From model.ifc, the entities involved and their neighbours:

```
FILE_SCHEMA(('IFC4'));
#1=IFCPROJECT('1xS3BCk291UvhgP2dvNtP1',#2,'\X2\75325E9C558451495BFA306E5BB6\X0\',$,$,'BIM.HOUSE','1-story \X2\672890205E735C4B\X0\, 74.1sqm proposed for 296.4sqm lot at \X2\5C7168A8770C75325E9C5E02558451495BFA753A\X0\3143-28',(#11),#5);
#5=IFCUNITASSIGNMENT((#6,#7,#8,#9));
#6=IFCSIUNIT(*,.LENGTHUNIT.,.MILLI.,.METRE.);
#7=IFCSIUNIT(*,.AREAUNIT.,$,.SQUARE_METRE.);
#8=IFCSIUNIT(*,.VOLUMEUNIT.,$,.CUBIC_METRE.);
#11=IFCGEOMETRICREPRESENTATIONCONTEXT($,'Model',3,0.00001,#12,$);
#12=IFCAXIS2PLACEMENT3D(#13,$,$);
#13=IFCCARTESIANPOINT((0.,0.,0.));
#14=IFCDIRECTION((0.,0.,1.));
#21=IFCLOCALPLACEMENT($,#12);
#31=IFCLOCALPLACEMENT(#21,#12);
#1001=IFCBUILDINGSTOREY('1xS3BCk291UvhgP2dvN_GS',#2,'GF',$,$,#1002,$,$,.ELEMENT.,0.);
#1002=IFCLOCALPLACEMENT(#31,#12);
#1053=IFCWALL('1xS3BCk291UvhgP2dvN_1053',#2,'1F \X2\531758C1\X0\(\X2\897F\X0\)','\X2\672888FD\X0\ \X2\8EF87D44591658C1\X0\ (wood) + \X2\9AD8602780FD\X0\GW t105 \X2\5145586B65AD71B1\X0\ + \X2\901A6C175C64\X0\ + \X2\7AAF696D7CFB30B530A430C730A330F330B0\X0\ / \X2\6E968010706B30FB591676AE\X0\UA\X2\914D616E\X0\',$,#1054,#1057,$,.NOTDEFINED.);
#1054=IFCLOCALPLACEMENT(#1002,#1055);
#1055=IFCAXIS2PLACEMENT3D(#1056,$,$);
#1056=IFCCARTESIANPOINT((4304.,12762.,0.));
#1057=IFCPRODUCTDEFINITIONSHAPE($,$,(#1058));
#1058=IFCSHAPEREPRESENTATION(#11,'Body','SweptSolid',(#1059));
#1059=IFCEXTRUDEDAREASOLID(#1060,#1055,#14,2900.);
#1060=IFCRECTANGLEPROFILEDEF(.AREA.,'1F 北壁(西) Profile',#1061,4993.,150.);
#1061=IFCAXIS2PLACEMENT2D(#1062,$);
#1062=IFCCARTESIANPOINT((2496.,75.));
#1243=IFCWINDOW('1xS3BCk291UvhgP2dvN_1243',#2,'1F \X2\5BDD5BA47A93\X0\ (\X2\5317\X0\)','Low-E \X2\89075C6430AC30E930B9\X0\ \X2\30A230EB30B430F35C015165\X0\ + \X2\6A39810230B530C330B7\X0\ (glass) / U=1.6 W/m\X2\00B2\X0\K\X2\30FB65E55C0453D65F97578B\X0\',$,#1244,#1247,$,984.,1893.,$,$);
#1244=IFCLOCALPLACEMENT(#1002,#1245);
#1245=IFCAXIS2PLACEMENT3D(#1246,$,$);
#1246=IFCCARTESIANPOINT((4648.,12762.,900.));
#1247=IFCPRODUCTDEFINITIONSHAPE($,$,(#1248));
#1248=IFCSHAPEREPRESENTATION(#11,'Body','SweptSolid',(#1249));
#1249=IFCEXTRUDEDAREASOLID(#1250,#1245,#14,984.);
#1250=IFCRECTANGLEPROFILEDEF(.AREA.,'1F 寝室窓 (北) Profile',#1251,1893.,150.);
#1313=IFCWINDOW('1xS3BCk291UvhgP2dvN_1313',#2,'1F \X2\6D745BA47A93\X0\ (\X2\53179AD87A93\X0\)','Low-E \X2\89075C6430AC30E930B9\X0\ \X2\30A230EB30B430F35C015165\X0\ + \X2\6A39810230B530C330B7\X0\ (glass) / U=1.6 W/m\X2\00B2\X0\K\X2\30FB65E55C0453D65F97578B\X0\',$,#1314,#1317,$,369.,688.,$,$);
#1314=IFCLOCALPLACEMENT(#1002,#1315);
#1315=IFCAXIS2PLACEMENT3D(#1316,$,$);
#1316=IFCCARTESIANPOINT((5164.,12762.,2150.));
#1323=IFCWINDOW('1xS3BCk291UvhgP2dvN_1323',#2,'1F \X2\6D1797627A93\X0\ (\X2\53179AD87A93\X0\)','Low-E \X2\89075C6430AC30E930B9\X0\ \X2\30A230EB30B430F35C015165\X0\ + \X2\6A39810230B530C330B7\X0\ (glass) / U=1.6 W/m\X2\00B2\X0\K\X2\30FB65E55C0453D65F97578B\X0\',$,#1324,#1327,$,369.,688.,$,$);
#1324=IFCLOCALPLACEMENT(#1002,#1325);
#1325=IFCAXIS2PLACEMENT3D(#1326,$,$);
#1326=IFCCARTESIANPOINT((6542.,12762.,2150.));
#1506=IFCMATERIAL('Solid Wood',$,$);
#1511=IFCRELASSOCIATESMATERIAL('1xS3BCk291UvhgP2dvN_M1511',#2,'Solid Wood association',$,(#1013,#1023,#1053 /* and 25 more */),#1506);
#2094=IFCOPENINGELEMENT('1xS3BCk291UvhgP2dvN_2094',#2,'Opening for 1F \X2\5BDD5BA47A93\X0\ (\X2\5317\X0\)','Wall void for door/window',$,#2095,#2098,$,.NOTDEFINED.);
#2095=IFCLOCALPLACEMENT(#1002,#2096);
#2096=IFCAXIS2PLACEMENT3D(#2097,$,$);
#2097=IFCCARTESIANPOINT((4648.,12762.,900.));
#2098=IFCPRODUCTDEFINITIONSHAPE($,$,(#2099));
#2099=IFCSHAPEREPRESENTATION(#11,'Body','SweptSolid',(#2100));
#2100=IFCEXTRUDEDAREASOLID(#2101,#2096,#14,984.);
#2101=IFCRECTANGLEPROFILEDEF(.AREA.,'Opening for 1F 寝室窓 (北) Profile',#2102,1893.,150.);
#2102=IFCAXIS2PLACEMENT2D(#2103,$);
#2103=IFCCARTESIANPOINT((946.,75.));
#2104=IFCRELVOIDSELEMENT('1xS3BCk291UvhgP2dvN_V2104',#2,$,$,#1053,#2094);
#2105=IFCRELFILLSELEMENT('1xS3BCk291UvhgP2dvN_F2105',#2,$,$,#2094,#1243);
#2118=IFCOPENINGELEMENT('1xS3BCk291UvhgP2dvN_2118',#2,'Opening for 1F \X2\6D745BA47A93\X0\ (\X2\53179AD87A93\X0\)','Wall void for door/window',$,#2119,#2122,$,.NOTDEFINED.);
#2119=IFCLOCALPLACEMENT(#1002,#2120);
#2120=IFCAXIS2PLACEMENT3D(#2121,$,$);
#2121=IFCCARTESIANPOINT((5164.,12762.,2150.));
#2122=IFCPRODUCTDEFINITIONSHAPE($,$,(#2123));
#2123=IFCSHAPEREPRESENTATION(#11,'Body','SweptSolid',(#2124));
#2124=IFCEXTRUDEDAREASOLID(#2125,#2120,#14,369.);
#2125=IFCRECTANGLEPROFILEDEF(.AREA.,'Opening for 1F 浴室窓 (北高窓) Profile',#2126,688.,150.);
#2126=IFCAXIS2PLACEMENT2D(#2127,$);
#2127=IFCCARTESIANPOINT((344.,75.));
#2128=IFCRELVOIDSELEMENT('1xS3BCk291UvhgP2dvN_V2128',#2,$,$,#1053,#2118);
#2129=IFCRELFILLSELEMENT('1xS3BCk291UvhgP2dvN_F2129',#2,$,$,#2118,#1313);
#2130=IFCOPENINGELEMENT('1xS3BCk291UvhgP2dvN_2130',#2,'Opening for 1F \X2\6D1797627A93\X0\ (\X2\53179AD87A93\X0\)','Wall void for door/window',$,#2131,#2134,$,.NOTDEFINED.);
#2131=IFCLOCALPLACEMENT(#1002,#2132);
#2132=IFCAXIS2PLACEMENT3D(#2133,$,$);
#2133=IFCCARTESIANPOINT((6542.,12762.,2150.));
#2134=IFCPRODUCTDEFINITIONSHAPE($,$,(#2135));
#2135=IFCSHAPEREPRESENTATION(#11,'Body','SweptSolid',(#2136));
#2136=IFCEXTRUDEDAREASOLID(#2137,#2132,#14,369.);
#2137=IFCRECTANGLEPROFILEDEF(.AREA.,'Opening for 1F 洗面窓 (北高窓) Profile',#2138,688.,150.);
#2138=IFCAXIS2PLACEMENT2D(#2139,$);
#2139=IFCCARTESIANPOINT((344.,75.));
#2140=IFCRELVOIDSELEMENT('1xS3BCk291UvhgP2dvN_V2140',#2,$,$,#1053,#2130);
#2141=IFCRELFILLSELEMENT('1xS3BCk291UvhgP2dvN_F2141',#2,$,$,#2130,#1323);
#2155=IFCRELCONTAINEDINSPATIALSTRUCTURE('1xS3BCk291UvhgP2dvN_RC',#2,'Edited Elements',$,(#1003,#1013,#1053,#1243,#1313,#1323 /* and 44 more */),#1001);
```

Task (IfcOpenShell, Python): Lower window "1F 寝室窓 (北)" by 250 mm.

```python
import numpy as np
import ifcopenshell
import ifcopenshell.api.geometry
import ifcopenshell.util.placement
import ifcopenshell.util.unit

model = ifcopenshell.open("model.ifc")
unit_scale = ifcopenshell.util.unit.calculate_unit_scale(model)

window = model.by_guid("1xS3BCk291UvhgP2dvN_1243")
opening = window.FillsVoids[0].RelatingOpeningElement
dz = -0.25 / unit_scale

shift = np.array([0.0, 0.0, dz])
# The window is not placed relative to its opening, so move both.
for product in (opening, window):
    matrix = ifcopenshell.util.placement.get_local_placement(product.ObjectPlacement)
    matrix[:3, 3] += shift
    ifcopenshell.api.geometry.edit_object_placement(model, product=product, matrix=matrix, is_si=False)

print(f"moved by {dz * unit_scale:+.3f} m")

model.write("model-out.ifc")
```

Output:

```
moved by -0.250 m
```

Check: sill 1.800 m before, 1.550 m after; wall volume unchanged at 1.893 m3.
